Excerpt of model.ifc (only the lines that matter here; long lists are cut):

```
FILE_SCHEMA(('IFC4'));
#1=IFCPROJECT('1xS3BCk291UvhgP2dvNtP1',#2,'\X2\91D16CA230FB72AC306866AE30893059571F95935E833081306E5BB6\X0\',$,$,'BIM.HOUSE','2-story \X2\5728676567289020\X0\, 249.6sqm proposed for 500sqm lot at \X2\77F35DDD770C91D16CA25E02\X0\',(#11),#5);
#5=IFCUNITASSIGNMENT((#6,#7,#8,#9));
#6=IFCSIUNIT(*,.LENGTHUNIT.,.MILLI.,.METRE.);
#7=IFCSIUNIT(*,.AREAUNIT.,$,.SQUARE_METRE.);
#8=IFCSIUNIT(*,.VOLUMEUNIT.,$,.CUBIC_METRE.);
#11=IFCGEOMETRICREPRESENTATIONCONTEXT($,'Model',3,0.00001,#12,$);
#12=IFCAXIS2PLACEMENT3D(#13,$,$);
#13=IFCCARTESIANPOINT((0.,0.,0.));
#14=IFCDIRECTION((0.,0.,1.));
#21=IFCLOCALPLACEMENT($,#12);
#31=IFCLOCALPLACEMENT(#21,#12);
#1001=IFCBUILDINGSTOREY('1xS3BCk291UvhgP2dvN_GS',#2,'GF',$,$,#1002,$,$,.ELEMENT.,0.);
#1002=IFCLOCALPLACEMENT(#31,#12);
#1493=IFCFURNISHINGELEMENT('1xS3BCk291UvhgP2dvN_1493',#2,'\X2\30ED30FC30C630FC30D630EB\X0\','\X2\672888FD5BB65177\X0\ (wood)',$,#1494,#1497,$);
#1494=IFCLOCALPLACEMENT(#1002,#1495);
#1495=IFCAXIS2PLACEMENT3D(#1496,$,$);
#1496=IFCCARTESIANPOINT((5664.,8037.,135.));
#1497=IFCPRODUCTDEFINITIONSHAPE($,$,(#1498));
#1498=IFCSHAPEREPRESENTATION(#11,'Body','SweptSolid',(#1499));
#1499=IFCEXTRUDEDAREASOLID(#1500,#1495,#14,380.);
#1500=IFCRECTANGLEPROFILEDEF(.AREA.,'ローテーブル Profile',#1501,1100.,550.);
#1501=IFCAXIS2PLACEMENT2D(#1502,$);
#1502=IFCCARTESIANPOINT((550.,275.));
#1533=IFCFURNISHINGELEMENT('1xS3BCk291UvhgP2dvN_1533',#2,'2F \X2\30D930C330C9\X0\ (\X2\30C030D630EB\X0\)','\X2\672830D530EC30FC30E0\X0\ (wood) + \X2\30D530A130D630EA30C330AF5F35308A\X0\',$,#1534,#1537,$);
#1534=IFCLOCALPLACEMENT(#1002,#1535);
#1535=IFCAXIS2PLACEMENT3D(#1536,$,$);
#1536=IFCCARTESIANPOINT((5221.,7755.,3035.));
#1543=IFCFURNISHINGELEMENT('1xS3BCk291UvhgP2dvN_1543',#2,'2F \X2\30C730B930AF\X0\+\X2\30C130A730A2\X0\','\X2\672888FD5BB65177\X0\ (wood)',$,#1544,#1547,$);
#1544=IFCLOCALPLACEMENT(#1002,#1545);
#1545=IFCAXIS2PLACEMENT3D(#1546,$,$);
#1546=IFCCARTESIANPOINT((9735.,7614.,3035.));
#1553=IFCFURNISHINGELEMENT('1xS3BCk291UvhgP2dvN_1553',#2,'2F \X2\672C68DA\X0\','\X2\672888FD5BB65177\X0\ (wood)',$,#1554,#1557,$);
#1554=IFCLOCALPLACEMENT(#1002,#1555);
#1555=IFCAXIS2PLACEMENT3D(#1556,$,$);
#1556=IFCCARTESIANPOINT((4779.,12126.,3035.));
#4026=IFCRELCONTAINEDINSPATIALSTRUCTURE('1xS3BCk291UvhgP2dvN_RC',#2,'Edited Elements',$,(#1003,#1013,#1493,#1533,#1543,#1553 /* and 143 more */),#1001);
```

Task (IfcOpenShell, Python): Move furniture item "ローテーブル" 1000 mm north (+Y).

```python
import ifcopenshell
import ifcopenshell.api.geometry
import ifcopenshell.util.placement

model = ifcopenshell.open("model.ifc")

item = model.by_guid("1xS3BCk291UvhgP2dvN_1493")
matrix = ifcopenshell.util.placement.get_local_placement(item.ObjectPlacement)
matrix[1, 3] += 1000.0
ifcopenshell.api.geometry.edit_object_placement(model, product=item, matrix=matrix, is_si=False)

print(ifcopenshell.util.placement.get_local_placement(item.ObjectPlacement).round(3) + 0.0)

model.write("model_updated.ifc")
```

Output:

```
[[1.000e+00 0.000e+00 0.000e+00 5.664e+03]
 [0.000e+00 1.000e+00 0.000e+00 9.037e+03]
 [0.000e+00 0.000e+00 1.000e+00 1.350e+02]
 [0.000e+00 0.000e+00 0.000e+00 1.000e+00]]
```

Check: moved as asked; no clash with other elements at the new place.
